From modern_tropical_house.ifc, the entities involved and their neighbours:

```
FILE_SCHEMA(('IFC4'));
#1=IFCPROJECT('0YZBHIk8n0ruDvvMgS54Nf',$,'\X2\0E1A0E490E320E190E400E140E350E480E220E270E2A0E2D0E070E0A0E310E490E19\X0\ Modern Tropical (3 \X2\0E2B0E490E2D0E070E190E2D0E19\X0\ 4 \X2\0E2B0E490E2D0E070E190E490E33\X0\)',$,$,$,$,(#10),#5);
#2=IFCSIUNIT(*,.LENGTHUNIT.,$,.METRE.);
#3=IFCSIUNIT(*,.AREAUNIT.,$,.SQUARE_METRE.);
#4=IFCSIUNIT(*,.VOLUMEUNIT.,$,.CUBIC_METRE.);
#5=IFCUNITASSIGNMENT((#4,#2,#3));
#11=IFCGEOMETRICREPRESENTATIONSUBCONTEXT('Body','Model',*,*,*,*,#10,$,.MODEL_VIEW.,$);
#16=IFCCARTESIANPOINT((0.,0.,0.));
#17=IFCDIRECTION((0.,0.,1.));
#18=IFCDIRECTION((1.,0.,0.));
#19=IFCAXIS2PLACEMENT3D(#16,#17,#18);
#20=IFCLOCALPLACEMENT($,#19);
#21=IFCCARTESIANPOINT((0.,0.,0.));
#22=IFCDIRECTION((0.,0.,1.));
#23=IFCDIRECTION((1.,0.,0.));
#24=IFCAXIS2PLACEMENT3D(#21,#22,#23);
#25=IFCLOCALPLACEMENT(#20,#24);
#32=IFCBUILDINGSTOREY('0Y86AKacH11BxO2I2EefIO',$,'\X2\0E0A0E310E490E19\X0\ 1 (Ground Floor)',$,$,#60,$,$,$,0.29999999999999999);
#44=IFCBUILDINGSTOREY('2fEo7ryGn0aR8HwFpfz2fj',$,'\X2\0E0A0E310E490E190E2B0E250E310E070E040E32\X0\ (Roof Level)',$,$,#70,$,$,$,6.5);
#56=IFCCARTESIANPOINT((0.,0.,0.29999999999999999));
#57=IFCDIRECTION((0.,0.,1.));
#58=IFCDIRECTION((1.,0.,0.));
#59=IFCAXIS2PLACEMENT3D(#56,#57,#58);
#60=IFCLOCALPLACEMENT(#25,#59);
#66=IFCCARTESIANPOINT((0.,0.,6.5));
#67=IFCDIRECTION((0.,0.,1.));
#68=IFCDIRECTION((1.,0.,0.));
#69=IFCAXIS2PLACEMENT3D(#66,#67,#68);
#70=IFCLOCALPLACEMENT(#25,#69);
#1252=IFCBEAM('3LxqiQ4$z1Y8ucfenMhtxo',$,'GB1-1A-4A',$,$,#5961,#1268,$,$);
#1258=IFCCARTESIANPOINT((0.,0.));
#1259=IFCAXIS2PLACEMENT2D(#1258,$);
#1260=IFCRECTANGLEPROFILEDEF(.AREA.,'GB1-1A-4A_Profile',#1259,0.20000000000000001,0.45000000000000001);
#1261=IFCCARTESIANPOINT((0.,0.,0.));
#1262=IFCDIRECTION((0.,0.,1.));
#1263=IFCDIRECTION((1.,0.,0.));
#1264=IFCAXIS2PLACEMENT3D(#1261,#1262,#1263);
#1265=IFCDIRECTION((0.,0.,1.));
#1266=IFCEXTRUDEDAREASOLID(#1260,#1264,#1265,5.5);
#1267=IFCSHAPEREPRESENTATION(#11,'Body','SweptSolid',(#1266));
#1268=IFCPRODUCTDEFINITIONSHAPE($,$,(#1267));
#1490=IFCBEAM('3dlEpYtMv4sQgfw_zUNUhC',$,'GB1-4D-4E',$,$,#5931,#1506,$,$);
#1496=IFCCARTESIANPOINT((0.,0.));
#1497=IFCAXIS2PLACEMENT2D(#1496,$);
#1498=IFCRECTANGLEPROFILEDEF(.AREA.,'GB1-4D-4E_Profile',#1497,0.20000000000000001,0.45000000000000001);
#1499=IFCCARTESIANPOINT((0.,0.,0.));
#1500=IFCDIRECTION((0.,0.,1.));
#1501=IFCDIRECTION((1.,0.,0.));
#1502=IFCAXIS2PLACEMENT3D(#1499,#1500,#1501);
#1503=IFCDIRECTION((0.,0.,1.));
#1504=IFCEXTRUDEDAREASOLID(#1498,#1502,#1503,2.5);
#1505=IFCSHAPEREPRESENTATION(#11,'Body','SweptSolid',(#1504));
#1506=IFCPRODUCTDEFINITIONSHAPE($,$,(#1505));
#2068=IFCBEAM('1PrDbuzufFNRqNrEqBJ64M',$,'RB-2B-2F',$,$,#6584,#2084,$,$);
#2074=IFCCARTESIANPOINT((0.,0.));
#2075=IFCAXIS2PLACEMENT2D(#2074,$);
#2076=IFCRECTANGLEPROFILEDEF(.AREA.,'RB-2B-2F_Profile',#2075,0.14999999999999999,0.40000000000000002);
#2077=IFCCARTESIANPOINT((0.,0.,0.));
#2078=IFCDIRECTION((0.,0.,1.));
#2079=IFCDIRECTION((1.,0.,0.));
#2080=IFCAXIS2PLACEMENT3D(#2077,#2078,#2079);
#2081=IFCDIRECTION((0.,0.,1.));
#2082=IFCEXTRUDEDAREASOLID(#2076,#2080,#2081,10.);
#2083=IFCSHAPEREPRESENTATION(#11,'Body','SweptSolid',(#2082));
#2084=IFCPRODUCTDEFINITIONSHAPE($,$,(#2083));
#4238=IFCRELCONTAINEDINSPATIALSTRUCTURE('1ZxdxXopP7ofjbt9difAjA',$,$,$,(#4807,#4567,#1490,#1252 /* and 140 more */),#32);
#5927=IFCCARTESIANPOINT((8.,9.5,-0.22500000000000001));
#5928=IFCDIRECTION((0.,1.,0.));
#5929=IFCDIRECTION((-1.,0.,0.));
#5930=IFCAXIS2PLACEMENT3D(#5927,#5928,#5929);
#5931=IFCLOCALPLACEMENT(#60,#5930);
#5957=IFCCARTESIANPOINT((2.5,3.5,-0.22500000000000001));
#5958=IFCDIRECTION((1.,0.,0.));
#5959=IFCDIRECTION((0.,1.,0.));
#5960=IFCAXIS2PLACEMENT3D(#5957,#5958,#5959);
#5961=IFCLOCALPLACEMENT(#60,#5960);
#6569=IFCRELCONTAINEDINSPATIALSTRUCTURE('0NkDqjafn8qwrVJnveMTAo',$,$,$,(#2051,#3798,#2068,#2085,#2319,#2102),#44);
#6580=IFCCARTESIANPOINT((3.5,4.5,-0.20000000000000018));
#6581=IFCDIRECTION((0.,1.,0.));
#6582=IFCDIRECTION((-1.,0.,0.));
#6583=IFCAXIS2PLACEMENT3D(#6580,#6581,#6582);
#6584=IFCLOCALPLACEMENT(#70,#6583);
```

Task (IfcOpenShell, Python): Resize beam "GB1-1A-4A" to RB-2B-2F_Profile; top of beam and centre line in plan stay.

```python
import ifcopenshell
import ifcopenshell.util.element
import ifcopenshell.util.representation

model = ifcopenshell.open("modern_tropical_house.ifc")

member = model.by_id(1252)
source = next(p for p in model.by_type("IfcRectangleProfileDef") if p.ProfileName == "RB-2B-2F_Profile")

body = ifcopenshell.util.representation.get_representation(member, "Model", "Body")
solid = body.Items[0]
old_profile = solid.SweptArea

# Copy the section's sizes but keep this member's own profile position.
profile = ifcopenshell.util.element.copy(model, source)
# Profiles are centred, so shift by half the change in depth to hold the top.
shift = (old_profile.YDim - profile.YDim) / 2
x, y = old_profile.Position.Location.Coordinates
up = (0.0, 1.0)  # upwards, in the solid's own plane
location = model.createIfcCartesianPoint((x + up[0] * shift, y + up[1] * shift))
profile.Position = model.createIfcAxis2Placement2D(location, old_profile.Position.RefDirection)
solid.SweptArea = profile
if not model.get_total_inverses(old_profile):
    ifcopenshell.util.element.remove_deep2(model, old_profile)

print(solid.SweptArea)

model.write("modern_tropical_house_v2.ifc")
```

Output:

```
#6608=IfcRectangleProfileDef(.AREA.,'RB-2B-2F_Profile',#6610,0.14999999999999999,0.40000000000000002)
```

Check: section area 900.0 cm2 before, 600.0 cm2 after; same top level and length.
